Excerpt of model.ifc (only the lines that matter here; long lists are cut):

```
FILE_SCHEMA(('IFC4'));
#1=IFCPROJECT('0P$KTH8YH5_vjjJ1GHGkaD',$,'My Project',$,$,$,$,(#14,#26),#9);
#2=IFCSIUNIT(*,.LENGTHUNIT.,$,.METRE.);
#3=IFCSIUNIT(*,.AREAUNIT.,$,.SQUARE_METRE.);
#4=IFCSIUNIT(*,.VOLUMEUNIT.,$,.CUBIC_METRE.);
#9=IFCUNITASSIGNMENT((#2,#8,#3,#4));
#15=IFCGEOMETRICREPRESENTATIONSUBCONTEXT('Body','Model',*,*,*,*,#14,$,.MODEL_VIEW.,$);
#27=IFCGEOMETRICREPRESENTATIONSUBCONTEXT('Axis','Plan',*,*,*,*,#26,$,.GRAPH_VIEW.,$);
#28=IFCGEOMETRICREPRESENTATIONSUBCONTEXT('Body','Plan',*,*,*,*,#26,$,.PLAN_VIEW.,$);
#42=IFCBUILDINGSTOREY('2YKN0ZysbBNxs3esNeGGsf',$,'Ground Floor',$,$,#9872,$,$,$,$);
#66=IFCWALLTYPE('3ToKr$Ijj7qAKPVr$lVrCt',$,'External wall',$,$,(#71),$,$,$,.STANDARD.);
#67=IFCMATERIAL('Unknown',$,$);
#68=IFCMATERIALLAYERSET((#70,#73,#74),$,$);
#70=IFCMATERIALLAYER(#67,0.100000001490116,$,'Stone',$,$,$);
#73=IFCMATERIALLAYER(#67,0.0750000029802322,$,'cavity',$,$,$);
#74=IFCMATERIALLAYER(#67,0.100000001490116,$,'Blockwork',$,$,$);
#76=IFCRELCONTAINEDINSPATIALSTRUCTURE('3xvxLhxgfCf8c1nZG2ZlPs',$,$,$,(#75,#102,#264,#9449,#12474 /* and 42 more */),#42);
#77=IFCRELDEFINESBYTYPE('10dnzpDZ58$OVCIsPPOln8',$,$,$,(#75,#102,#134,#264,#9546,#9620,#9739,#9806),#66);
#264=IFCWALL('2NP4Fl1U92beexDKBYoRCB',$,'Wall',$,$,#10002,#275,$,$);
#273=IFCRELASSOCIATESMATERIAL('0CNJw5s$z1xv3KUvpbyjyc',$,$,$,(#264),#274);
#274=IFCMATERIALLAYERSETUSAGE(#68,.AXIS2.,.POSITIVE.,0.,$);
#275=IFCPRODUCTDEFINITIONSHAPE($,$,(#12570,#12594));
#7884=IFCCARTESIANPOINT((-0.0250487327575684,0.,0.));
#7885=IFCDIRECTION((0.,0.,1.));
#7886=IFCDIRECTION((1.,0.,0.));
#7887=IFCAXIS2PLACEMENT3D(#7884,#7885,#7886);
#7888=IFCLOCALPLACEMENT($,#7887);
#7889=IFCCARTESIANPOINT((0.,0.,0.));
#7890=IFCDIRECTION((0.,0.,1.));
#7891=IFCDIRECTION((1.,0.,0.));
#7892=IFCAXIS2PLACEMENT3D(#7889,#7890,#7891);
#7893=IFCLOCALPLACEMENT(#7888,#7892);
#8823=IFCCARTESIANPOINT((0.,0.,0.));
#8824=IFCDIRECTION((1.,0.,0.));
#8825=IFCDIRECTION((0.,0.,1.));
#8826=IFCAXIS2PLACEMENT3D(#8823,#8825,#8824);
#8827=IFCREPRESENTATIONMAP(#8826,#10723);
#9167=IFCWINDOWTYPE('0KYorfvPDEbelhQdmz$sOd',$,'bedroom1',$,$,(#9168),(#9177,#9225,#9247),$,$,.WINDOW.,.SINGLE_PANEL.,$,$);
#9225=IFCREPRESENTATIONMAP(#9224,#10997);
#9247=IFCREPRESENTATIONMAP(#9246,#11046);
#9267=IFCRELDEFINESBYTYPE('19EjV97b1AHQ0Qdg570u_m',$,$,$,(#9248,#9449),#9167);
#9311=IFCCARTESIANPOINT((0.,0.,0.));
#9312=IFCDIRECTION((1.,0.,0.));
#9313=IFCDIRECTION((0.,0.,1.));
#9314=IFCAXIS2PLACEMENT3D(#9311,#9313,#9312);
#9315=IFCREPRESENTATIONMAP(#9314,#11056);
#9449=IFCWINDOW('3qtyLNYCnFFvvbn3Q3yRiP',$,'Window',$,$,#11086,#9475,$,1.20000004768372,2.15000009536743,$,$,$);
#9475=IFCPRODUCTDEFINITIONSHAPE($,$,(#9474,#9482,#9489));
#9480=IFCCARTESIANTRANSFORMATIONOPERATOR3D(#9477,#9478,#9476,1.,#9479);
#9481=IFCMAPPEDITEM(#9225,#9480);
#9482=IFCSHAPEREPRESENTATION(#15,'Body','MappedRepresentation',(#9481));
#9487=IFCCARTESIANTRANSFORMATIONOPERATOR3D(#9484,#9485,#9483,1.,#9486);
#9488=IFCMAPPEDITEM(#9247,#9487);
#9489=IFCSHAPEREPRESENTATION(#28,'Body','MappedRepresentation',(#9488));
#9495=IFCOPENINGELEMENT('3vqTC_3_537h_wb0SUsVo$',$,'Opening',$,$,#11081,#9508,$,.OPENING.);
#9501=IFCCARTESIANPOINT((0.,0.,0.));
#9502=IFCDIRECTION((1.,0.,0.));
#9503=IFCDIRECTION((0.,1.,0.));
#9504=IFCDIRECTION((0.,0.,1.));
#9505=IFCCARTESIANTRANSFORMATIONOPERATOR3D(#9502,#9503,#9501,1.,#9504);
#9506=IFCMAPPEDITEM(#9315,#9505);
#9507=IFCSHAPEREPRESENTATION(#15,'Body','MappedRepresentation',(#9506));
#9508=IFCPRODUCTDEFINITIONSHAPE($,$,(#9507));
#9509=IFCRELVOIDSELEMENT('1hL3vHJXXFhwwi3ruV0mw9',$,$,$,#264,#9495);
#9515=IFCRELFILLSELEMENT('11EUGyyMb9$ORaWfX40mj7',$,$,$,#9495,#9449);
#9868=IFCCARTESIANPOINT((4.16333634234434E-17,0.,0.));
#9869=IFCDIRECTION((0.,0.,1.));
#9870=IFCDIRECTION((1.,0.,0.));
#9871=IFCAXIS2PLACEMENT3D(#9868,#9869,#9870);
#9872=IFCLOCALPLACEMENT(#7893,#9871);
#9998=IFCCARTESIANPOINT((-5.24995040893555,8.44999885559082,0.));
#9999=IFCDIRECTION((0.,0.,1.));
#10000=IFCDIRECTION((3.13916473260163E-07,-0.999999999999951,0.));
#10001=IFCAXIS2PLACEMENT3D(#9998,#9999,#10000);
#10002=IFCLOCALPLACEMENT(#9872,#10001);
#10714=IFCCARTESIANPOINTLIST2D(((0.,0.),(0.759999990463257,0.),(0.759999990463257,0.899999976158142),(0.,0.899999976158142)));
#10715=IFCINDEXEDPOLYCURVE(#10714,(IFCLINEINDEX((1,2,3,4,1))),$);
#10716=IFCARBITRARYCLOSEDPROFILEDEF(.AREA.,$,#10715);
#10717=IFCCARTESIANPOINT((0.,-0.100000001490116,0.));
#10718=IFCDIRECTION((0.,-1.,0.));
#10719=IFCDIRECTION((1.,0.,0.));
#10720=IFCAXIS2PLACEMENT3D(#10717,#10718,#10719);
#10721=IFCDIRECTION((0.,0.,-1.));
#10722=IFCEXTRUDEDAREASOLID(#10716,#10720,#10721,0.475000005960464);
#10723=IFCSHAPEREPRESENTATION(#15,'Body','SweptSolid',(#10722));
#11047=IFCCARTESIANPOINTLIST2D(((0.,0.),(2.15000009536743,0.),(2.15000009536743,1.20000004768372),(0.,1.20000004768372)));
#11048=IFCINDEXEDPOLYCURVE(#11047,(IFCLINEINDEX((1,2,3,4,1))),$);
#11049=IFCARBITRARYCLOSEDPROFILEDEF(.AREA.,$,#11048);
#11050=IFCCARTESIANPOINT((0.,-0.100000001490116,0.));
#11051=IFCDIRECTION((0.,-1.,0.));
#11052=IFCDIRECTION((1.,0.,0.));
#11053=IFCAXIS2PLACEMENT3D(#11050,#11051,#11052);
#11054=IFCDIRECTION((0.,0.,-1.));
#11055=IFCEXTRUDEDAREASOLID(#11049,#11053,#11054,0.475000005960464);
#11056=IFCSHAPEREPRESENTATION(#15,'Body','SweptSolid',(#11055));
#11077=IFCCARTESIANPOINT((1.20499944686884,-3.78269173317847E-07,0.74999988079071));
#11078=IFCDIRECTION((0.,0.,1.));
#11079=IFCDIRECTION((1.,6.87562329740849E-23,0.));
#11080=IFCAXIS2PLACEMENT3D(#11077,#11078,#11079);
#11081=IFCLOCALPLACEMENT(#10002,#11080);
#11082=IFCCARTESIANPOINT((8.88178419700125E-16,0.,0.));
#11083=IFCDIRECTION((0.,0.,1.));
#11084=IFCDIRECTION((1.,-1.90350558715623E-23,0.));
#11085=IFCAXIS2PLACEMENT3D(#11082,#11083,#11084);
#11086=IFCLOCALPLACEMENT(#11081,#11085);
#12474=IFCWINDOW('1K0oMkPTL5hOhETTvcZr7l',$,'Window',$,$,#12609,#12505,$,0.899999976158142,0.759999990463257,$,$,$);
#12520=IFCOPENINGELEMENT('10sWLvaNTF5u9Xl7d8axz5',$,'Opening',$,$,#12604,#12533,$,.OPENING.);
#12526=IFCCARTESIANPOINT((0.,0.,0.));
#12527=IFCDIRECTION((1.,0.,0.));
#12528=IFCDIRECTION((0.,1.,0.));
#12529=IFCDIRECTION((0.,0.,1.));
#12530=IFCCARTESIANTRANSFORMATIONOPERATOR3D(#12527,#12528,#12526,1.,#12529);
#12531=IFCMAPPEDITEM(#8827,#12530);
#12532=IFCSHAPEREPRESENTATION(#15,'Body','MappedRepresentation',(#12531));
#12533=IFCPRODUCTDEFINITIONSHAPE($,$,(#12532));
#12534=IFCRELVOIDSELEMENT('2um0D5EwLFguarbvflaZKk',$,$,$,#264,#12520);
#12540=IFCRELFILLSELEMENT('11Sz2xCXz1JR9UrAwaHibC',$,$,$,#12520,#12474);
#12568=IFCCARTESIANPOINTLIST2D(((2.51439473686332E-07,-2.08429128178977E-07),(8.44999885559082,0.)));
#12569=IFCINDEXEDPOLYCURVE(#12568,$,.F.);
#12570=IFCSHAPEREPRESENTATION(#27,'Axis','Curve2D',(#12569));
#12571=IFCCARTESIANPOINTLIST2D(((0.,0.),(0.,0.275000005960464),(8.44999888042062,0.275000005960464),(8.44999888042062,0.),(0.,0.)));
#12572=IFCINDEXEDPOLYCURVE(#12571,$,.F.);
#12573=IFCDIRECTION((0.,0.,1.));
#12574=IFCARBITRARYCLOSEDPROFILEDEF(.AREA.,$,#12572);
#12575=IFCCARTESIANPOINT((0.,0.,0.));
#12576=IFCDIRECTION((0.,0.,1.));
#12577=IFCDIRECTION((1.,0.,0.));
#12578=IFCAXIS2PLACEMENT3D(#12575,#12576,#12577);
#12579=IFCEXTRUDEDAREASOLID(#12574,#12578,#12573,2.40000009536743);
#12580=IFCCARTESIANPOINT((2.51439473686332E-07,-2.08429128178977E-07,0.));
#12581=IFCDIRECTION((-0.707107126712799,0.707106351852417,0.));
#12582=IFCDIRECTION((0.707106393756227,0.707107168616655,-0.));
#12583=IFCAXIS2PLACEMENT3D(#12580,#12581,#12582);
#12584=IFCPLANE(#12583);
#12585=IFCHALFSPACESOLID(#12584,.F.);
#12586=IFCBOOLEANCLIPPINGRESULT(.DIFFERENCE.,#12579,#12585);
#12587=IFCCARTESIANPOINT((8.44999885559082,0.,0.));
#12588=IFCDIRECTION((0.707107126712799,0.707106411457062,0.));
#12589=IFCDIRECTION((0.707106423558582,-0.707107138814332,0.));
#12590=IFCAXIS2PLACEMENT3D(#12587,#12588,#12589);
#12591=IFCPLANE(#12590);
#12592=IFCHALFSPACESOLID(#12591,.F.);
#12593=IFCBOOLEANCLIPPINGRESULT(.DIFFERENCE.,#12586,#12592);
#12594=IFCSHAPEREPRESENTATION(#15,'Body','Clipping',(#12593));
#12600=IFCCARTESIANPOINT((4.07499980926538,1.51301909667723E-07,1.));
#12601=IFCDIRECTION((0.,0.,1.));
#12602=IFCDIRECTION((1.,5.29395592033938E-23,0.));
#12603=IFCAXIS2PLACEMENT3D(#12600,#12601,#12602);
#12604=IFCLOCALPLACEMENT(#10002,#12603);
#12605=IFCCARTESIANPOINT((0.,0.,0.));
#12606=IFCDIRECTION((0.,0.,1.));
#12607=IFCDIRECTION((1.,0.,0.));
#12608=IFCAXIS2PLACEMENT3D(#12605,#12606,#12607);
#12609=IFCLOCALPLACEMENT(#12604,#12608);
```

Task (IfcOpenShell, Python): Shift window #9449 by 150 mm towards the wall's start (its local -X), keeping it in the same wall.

```python
import ifcopenshell
import ifcopenshell.api.geometry
import ifcopenshell.util.placement
import ifcopenshell.util.unit

model = ifcopenshell.open("model.ifc")
unit_scale = ifcopenshell.util.unit.calculate_unit_scale(model)

window = model.by_id(9449)
opening = window.FillsVoids[0].RelatingOpeningElement
wall = opening.VoidsElements[0].RelatingBuildingElement

wall_matrix = ifcopenshell.util.placement.get_local_placement(wall.ObjectPlacement)
shift = wall_matrix[:3, 0] * -0.15 / unit_scale
before = ifcopenshell.util.placement.get_local_placement(window.ObjectPlacement)[:3, 3].copy()

# The window is placed relative to its opening, so it follows when the opening moves.
matrix = ifcopenshell.util.placement.get_local_placement(opening.ObjectPlacement)
matrix[:3, 3] += shift
ifcopenshell.api.geometry.edit_object_placement(
    model, product=opening, matrix=matrix, is_si=False, should_transform_children=True
)

after = ifcopenshell.util.placement.get_local_placement(window.ObjectPlacement)[:3, 3]
print("window moved by", (after - before).round(3) + 0.0)

model.write("model_v2.ifc")
```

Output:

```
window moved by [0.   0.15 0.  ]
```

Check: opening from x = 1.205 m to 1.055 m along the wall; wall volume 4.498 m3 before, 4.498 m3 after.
